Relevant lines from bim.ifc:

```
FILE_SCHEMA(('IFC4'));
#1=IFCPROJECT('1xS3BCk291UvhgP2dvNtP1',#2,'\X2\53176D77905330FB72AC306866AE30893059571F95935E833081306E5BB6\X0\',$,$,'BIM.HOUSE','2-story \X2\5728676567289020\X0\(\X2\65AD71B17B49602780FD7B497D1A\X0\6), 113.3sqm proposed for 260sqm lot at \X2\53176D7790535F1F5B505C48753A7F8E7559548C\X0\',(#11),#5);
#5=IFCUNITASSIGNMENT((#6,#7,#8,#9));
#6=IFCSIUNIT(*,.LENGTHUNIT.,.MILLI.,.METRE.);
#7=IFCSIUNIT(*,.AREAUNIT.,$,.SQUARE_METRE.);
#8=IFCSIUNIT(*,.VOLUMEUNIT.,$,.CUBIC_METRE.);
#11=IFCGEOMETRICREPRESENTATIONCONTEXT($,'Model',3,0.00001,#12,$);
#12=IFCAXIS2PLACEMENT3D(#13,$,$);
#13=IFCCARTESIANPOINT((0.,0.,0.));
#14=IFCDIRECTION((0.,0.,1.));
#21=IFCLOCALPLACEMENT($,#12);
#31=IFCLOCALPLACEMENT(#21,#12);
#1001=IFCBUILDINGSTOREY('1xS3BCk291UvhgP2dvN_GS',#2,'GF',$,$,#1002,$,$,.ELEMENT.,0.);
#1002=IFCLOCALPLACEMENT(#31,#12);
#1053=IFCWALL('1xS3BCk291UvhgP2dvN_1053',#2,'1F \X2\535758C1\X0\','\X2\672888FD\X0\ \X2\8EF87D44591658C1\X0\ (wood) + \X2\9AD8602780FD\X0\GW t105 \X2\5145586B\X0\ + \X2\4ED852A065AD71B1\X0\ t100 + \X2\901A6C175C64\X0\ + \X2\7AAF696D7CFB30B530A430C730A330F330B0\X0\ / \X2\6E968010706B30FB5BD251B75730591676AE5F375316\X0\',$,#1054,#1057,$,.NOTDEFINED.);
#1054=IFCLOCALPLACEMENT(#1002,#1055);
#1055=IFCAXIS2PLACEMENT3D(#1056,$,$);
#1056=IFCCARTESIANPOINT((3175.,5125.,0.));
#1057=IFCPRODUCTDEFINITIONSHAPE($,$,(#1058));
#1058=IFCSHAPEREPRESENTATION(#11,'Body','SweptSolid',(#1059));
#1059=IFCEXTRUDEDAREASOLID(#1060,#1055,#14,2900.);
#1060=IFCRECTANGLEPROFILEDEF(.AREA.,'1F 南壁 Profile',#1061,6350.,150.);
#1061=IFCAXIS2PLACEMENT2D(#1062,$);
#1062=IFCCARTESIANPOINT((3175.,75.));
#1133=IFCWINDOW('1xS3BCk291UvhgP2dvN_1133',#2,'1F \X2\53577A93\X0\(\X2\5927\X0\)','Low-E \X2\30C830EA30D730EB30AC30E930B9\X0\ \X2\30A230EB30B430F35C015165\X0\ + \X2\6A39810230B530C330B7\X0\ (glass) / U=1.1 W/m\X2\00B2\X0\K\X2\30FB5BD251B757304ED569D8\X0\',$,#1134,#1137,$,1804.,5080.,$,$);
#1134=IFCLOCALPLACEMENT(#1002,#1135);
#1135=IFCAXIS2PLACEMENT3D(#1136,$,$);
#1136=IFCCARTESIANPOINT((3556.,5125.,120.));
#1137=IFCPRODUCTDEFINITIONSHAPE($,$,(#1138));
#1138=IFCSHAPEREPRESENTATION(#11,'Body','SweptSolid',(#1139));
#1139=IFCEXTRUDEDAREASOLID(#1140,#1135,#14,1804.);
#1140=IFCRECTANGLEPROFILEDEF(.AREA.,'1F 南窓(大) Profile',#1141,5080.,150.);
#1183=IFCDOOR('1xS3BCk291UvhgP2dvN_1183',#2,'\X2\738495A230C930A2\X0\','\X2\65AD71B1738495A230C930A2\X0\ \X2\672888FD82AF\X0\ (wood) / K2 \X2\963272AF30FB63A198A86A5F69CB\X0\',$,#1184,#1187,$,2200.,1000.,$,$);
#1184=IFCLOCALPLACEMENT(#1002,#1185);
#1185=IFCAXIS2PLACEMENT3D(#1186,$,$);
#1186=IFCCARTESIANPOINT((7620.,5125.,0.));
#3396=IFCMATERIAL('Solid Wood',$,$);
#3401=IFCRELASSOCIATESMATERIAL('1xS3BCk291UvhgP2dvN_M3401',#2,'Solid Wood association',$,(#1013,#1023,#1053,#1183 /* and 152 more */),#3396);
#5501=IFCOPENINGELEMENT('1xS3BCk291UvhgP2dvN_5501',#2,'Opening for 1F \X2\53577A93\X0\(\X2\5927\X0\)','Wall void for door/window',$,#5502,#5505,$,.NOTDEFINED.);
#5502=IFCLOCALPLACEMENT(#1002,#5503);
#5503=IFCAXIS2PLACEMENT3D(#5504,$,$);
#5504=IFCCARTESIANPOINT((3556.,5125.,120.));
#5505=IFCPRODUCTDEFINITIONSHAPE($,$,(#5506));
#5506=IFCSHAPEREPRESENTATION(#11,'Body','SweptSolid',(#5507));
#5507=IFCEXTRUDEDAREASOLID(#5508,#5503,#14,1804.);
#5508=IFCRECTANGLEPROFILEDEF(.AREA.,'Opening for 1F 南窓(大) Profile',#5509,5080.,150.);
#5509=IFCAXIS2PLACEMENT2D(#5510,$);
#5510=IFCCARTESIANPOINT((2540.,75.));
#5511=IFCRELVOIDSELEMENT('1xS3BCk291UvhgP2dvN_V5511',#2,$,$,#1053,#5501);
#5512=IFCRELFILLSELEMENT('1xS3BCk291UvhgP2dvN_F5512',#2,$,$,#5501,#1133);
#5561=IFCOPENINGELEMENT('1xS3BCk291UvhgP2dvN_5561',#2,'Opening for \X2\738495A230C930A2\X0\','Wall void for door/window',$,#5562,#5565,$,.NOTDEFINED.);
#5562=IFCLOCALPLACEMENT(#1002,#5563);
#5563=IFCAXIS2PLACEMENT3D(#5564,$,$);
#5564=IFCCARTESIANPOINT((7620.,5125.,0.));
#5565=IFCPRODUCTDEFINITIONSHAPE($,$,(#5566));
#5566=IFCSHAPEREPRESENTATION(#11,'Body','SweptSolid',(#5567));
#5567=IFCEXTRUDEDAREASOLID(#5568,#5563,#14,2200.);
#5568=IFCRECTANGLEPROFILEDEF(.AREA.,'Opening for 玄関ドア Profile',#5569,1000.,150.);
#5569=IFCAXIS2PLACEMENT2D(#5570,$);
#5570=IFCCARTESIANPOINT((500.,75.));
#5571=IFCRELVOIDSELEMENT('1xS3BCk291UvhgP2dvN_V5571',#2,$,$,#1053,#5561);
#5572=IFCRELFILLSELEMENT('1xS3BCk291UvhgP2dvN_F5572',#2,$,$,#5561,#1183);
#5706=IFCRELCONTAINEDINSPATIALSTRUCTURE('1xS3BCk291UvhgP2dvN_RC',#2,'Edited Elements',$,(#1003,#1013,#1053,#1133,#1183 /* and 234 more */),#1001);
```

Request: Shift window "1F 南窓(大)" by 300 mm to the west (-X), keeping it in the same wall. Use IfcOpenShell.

```python
import ifcopenshell
import ifcopenshell.api.geometry
import ifcopenshell.util.placement
import ifcopenshell.util.unit

model = ifcopenshell.open("bim.ifc")
unit_scale = ifcopenshell.util.unit.calculate_unit_scale(model)

window = model.by_guid("1xS3BCk291UvhgP2dvN_1133")
opening = window.FillsVoids[0].RelatingOpeningElement
wall = opening.VoidsElements[0].RelatingBuildingElement

wall_matrix = ifcopenshell.util.placement.get_local_placement(wall.ObjectPlacement)
shift = wall_matrix[:3, 0] * -0.3 / unit_scale
before = ifcopenshell.util.placement.get_local_placement(window.ObjectPlacement)[:3, 3].copy()

# The window is not placed relative to its opening, so move both.
for product in (opening, window):
    matrix = ifcopenshell.util.placement.get_local_placement(product.ObjectPlacement)
    matrix[:3, 3] += shift
    ifcopenshell.api.geometry.edit_object_placement(model, product=product, matrix=matrix, is_si=False)

after = ifcopenshell.util.placement.get_local_placement(window.ObjectPlacement)[:3, 3]
print("window moved by", (after - before).round(3) + 0.0)

model.write("bim_rev.ifc")
```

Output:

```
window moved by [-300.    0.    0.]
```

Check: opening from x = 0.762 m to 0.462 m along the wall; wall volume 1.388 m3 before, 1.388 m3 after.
